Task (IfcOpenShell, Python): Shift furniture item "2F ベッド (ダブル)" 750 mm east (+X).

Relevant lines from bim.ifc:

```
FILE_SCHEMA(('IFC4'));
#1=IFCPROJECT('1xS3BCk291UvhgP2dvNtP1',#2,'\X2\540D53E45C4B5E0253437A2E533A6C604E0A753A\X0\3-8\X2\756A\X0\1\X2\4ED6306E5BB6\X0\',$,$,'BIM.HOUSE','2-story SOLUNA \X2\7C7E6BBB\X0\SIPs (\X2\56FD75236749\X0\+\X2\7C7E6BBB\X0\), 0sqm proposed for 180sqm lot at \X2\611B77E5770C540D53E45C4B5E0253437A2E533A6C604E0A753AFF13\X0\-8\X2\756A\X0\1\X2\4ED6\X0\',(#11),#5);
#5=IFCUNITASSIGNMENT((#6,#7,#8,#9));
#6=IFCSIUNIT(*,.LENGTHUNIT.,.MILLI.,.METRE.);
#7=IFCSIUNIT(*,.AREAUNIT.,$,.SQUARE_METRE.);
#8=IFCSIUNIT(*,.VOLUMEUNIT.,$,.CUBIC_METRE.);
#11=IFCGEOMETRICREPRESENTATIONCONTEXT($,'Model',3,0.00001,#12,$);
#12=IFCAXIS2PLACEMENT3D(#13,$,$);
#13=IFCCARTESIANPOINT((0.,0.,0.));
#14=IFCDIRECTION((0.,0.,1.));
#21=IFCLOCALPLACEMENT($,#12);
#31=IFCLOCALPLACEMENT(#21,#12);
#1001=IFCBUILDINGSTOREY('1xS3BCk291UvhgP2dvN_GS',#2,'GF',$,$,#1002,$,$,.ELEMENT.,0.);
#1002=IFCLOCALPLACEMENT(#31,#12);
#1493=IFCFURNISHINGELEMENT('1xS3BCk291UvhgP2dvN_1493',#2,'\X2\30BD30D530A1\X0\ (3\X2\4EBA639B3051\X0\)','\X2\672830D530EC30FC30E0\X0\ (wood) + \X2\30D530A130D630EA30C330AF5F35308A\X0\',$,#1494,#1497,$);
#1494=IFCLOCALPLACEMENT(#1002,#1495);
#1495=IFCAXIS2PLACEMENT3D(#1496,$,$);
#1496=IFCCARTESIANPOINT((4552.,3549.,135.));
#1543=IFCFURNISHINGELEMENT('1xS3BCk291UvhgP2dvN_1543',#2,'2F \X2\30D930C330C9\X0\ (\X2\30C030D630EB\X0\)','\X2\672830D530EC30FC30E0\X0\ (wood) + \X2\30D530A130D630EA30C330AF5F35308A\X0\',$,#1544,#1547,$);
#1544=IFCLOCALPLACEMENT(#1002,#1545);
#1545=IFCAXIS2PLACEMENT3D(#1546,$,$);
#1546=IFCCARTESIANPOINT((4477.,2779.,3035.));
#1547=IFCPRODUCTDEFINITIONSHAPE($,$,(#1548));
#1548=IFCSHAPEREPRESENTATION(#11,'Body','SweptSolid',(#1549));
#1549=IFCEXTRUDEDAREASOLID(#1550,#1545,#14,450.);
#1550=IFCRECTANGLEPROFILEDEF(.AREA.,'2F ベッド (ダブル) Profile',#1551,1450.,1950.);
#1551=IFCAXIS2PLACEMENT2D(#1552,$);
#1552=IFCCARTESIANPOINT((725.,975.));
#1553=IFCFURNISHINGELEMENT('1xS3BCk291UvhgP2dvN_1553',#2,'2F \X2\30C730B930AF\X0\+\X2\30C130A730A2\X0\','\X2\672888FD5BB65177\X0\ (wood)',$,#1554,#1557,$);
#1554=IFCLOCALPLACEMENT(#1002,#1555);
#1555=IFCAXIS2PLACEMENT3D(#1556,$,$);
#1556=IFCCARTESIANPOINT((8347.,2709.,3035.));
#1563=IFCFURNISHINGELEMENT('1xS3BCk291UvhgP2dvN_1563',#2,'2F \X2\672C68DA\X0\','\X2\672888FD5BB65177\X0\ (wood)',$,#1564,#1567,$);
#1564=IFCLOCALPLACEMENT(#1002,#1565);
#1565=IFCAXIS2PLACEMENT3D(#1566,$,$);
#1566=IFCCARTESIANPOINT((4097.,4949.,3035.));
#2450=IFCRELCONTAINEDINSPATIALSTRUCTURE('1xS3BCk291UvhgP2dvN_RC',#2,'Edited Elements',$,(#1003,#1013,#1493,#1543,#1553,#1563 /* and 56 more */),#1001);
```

```python
import ifcopenshell
import ifcopenshell.api.geometry
import ifcopenshell.util.placement
import ifcopenshell.util.unit

model = ifcopenshell.open("bim.ifc")
unit_scale = ifcopenshell.util.unit.calculate_unit_scale(model)

item = model.by_guid("1xS3BCk291UvhgP2dvN_1543")
matrix = ifcopenshell.util.placement.get_local_placement(item.ObjectPlacement)
matrix[0, 3] += 0.75 / unit_scale
ifcopenshell.api.geometry.edit_object_placement(model, product=item, matrix=matrix, is_si=False)

print(ifcopenshell.util.placement.get_local_placement(item.ObjectPlacement).round(3) + 0.0)

model.write("bim-out.ifc")
```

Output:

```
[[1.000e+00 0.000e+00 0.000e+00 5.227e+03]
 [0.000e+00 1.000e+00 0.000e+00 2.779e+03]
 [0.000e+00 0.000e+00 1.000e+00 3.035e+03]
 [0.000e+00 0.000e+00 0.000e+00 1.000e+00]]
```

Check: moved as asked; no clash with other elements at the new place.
